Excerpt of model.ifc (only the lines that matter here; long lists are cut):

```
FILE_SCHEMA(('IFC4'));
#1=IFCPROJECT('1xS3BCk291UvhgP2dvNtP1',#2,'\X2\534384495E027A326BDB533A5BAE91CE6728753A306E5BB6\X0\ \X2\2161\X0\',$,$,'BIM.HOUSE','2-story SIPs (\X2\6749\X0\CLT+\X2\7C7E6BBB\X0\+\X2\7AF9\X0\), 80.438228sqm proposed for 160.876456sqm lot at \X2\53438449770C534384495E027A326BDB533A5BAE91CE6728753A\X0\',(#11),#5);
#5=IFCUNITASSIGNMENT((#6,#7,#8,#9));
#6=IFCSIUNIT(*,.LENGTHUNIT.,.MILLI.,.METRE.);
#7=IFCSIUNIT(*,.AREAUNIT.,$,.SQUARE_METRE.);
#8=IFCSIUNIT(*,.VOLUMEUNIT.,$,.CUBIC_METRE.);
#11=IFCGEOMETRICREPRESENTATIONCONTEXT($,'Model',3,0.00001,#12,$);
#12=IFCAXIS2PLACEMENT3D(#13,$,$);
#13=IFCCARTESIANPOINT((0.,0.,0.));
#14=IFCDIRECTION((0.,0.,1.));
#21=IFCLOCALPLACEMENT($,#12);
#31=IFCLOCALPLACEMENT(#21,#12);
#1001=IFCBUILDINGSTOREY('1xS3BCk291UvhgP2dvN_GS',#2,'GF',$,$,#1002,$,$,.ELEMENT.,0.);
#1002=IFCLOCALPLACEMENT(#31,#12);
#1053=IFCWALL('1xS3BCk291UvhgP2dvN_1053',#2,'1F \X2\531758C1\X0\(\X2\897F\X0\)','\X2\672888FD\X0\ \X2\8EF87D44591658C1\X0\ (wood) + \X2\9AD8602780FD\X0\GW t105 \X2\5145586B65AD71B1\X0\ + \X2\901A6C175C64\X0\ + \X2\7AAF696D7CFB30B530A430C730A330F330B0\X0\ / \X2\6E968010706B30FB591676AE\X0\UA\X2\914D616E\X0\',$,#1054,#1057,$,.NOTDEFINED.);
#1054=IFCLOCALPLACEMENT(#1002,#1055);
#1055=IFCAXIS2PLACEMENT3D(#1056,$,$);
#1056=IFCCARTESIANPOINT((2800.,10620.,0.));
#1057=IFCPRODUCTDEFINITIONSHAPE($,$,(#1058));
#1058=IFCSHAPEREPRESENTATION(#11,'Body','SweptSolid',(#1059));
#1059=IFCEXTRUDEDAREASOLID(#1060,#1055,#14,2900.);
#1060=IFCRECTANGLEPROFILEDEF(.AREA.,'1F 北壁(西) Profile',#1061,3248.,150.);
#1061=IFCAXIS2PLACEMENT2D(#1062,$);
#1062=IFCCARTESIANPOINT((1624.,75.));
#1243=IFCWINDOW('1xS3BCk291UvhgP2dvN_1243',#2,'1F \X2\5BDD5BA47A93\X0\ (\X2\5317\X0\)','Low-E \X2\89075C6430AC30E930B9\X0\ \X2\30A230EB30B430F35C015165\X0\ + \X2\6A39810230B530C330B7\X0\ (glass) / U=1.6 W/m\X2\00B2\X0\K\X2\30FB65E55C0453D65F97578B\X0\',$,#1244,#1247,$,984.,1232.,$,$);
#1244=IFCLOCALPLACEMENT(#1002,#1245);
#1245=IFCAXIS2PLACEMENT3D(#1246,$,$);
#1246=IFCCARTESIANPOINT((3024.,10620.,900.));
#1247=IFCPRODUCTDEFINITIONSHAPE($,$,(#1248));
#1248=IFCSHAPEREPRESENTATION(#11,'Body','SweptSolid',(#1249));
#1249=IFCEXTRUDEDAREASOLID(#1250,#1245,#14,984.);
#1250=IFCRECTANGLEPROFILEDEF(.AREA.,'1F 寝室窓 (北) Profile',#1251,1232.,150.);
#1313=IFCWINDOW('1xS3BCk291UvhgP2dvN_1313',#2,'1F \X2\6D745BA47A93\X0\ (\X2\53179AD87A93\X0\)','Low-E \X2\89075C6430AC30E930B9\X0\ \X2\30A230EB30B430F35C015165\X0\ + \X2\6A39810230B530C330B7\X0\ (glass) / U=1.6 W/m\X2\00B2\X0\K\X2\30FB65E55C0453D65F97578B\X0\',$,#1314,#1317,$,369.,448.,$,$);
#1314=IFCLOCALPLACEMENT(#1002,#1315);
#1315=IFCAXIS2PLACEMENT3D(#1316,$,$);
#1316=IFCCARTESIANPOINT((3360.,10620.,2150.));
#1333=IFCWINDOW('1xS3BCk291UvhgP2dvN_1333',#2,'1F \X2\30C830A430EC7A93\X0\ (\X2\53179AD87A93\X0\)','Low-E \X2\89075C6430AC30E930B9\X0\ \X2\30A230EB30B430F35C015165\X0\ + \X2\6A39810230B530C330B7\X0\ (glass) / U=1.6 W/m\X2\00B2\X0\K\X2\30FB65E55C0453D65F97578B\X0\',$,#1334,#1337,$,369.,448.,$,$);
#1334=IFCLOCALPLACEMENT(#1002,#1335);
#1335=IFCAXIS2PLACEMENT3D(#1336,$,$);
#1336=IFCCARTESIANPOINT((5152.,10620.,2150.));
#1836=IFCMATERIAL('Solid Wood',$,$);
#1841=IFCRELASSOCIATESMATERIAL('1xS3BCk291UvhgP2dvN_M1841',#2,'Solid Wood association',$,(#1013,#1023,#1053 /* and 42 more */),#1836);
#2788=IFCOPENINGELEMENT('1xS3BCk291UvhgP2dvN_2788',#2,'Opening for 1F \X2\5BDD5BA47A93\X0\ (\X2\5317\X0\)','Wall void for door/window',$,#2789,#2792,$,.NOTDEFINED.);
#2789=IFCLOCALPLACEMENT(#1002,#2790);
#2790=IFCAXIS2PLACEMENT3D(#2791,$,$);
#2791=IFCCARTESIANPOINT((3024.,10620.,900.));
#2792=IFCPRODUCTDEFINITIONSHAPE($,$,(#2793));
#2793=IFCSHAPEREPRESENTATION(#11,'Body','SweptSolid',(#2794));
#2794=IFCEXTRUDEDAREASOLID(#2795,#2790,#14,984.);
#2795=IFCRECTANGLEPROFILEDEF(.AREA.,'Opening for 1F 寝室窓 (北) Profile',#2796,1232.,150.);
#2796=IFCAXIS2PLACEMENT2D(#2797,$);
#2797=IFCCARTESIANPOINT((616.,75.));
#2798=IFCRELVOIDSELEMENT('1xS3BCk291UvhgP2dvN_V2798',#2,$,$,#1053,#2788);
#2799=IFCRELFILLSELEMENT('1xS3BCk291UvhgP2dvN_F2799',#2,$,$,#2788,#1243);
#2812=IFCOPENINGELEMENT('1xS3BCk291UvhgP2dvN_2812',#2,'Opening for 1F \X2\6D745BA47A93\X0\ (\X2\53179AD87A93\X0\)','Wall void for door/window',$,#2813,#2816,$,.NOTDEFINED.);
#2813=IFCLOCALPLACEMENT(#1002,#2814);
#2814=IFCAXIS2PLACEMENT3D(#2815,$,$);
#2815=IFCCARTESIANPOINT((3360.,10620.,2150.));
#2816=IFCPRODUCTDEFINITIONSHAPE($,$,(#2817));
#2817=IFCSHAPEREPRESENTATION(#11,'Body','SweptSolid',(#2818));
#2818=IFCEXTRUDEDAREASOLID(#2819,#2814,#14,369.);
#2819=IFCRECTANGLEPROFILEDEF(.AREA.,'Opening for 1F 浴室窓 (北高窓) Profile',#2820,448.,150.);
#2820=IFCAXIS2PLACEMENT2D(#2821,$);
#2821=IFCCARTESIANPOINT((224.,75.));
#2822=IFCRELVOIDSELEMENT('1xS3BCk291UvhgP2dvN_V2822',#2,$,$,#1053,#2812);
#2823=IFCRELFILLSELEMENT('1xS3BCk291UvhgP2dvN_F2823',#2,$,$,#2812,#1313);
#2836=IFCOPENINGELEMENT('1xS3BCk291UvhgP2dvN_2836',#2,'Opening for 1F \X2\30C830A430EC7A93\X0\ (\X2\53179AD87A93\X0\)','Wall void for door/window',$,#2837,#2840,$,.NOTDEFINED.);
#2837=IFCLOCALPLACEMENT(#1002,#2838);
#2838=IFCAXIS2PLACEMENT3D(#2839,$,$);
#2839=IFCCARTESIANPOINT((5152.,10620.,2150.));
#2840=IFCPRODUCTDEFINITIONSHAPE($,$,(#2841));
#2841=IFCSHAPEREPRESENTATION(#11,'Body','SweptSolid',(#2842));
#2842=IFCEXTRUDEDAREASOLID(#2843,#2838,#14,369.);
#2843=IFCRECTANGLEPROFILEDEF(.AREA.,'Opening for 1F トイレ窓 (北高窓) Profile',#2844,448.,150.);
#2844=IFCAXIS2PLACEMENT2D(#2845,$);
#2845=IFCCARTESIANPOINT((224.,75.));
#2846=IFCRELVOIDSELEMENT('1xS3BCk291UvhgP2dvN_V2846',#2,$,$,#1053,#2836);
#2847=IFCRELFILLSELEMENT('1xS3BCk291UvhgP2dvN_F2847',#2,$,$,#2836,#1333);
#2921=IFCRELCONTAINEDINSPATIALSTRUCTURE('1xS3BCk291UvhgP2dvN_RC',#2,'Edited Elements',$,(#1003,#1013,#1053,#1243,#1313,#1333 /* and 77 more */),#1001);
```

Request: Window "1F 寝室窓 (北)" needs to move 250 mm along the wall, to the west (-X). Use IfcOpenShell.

```python
import ifcopenshell
import ifcopenshell.api.geometry
import ifcopenshell.util.placement
import ifcopenshell.util.unit

model = ifcopenshell.open("model.ifc")
unit_scale = ifcopenshell.util.unit.calculate_unit_scale(model)

window = model.by_guid("1xS3BCk291UvhgP2dvN_1243")
opening = window.FillsVoids[0].RelatingOpeningElement
wall = opening.VoidsElements[0].RelatingBuildingElement

wall_matrix = ifcopenshell.util.placement.get_local_placement(wall.ObjectPlacement)
shift = wall_matrix[:3, 0] * -0.25 / unit_scale
before = ifcopenshell.util.placement.get_local_placement(window.ObjectPlacement)[:3, 3].copy()

# The window is not placed relative to its opening, so move both.
for product in (opening, window):
    matrix = ifcopenshell.util.placement.get_local_placement(product.ObjectPlacement)
    matrix[:3, 3] += shift
    ifcopenshell.api.geometry.edit_object_placement(model, product=product, matrix=matrix, is_si=False)

after = ifcopenshell.util.placement.get_local_placement(window.ObjectPlacement)[:3, 3]
print("window moved by", (after - before).round(3) + 0.0)

model.write("model_updated.ifc")
```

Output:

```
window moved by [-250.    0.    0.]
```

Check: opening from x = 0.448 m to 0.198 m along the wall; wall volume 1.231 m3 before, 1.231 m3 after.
